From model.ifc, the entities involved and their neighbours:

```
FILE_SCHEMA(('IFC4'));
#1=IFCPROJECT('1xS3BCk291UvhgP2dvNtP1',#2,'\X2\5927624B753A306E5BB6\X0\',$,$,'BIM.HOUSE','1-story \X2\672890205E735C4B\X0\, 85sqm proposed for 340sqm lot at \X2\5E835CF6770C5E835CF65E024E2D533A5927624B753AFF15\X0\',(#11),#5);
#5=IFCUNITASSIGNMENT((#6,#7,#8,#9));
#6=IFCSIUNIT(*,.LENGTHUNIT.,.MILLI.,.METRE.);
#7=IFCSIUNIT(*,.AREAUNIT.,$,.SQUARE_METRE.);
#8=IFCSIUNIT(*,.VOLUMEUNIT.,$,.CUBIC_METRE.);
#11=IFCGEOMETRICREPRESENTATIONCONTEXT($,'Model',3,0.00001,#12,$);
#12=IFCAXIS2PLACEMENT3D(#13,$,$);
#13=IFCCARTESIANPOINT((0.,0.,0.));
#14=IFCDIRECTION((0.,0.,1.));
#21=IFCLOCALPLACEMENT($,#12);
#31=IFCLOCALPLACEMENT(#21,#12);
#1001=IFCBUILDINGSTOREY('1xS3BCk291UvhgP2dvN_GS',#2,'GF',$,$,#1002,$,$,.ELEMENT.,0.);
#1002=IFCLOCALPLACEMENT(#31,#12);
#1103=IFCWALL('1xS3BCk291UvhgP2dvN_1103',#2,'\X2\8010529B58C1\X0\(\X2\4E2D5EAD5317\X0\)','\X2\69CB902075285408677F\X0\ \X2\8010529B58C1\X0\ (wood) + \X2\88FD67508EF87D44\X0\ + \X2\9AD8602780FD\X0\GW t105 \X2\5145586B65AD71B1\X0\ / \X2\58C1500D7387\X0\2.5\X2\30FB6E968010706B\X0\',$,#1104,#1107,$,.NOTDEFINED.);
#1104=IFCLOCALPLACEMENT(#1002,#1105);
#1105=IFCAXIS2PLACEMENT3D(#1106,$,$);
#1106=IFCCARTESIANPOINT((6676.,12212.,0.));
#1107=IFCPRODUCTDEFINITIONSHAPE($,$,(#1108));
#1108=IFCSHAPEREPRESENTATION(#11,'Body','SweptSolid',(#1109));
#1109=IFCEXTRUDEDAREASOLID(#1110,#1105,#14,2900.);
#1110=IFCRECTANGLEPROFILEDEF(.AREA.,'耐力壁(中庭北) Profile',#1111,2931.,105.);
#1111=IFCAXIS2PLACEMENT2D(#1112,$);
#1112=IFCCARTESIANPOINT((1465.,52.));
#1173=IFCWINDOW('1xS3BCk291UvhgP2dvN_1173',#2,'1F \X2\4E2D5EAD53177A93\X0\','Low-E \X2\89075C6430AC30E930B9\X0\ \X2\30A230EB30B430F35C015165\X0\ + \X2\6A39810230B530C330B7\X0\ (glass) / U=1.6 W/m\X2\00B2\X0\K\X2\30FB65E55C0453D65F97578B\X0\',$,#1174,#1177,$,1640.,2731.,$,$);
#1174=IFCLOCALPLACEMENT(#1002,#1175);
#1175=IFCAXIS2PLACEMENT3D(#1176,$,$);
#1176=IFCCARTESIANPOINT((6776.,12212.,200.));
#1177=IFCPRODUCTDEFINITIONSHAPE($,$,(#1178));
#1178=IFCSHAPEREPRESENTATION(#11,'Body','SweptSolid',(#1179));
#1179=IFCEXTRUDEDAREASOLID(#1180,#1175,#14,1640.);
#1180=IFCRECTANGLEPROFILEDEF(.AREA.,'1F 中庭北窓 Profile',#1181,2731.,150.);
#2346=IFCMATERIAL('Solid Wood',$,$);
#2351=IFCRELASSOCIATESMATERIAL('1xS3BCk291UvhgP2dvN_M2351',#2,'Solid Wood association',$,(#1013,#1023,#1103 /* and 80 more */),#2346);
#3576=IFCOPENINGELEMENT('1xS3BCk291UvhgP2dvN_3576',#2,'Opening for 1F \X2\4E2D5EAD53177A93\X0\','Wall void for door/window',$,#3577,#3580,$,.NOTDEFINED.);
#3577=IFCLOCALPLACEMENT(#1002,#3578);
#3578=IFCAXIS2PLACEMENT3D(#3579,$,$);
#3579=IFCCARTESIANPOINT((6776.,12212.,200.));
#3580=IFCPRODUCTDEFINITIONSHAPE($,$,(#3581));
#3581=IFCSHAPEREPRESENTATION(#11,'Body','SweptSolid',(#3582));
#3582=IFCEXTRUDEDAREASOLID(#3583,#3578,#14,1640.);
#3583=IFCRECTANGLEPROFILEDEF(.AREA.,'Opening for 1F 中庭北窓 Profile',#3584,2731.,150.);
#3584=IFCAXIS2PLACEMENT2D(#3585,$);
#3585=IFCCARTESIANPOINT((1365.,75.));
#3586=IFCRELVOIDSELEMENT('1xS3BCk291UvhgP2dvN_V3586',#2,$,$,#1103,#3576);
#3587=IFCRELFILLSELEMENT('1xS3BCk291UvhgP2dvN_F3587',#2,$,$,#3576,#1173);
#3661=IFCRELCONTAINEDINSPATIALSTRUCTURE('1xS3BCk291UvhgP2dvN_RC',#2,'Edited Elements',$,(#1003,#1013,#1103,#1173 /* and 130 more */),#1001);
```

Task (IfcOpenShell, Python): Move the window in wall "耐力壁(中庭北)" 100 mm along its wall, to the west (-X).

```python
import ifcopenshell
import ifcopenshell.api.geometry
import ifcopenshell.util.placement
import ifcopenshell.util.unit

model = ifcopenshell.open("model.ifc")
unit_scale = ifcopenshell.util.unit.calculate_unit_scale(model)

window = model.by_id(1173)
opening = window.FillsVoids[0].RelatingOpeningElement
wall = opening.VoidsElements[0].RelatingBuildingElement

wall_matrix = ifcopenshell.util.placement.get_local_placement(wall.ObjectPlacement)
shift = wall_matrix[:3, 0] * -0.1 / unit_scale
before = ifcopenshell.util.placement.get_local_placement(window.ObjectPlacement)[:3, 3].copy()

# The window is not placed relative to its opening, so move both.
for product in (opening, window):
    matrix = ifcopenshell.util.placement.get_local_placement(product.ObjectPlacement)
    matrix[:3, 3] += shift
    ifcopenshell.api.geometry.edit_object_placement(model, product=product, matrix=matrix, is_si=False)

after = ifcopenshell.util.placement.get_local_placement(window.ObjectPlacement)[:3, 3]
print("window moved by", (after - before).round(3) + 0.0)

model.write("model_v2.ifc")
```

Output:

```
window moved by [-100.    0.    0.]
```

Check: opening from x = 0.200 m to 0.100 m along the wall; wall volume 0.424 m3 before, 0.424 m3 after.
